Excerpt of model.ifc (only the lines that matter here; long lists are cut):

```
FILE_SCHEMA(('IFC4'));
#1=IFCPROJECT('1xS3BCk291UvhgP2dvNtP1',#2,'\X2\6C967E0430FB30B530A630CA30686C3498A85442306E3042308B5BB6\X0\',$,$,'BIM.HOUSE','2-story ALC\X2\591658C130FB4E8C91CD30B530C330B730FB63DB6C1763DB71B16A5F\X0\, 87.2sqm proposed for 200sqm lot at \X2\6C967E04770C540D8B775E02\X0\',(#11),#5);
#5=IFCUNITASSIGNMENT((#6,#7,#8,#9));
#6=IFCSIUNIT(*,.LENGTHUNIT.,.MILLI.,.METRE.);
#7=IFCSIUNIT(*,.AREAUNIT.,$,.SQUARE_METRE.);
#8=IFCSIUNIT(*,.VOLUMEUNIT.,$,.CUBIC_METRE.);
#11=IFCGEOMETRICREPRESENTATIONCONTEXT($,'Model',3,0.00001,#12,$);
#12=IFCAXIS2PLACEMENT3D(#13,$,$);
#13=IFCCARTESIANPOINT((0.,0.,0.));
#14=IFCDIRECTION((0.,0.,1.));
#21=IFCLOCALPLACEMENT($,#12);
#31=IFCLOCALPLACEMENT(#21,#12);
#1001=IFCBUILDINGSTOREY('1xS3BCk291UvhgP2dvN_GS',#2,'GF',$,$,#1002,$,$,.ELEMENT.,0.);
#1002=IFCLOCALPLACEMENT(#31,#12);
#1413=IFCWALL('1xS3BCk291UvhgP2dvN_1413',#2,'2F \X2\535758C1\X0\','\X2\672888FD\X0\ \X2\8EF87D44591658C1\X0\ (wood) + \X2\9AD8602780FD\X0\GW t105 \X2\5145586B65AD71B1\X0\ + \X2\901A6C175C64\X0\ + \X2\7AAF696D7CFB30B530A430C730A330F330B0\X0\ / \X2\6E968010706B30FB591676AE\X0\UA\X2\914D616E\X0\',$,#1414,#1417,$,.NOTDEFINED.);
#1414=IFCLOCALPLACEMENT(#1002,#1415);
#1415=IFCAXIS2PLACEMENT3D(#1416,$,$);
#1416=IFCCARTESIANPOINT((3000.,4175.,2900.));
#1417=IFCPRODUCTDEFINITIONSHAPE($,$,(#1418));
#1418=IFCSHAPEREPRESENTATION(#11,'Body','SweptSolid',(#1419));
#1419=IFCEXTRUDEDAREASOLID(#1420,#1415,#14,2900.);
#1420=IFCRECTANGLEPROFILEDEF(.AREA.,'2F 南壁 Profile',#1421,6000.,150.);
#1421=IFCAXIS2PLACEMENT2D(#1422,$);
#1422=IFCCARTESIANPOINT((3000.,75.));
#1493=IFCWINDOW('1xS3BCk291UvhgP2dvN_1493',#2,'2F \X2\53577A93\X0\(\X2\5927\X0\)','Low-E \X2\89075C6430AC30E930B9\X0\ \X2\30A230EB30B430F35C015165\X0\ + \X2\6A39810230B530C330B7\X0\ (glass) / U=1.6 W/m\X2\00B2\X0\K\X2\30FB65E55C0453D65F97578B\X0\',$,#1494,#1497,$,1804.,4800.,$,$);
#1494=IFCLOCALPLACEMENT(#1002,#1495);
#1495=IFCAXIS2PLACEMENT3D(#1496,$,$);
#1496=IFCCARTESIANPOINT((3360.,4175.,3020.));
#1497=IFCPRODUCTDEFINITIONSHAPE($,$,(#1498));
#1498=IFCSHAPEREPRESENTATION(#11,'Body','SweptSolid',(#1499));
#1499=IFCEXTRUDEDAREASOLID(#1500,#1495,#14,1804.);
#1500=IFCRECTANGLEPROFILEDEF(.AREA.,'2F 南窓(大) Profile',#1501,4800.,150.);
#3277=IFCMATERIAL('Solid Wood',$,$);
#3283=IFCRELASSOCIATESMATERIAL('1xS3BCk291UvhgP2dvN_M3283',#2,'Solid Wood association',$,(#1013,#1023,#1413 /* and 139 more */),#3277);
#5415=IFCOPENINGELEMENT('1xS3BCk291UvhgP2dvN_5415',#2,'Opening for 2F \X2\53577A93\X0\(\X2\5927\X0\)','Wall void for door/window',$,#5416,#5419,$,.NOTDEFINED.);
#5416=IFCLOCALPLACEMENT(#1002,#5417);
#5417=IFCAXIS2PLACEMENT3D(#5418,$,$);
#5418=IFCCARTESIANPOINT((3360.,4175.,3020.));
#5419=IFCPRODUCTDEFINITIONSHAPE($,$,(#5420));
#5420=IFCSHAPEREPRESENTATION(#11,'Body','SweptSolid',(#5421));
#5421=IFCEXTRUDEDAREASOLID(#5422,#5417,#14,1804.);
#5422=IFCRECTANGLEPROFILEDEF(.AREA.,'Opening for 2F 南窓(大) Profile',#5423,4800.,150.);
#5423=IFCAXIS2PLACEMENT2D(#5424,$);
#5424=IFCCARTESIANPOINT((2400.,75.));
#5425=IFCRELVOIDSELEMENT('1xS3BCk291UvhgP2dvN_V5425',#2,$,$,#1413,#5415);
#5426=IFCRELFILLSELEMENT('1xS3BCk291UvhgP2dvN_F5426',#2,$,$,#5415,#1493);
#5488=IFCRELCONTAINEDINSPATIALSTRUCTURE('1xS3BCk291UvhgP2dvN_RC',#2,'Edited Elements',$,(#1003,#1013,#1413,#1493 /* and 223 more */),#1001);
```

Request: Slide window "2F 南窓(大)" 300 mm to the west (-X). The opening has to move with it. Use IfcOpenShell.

```python
import ifcopenshell
import ifcopenshell.api.geometry
import ifcopenshell.util.placement

model = ifcopenshell.open("model.ifc")

window = model.by_guid("1xS3BCk291UvhgP2dvN_1493")
opening = window.FillsVoids[0].RelatingOpeningElement
wall = opening.VoidsElements[0].RelatingBuildingElement

wall_matrix = ifcopenshell.util.placement.get_local_placement(wall.ObjectPlacement)
shift = wall_matrix[:3, 0] * -300.0
before = ifcopenshell.util.placement.get_local_placement(window.ObjectPlacement)[:3, 3].copy()

# The window is not placed relative to its opening, so move both.
for product in (opening, window):
    matrix = ifcopenshell.util.placement.get_local_placement(product.ObjectPlacement)
    matrix[:3, 3] += shift
    ifcopenshell.api.geometry.edit_object_placement(model, product=product, matrix=matrix, is_si=False)

after = ifcopenshell.util.placement.get_local_placement(window.ObjectPlacement)[:3, 3]
print("window moved by", (after - before).round(3) + 0.0)

model.write("model_rev.ifc")
```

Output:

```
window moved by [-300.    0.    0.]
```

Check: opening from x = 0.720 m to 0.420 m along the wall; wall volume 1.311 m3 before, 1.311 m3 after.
